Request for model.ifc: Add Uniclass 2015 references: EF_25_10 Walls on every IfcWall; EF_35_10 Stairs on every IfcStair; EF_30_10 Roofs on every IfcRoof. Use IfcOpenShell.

First a look at what the model holds.

```python
import ifcopenshell

model = ifcopenshell.open("model.ifc")
print(model.schema)
print("classifications:", [c.Name for c in model.by_type("IfcClassification")])
for ifc_class in ("IfcDoor", "IfcRoof", "IfcStair", "IfcWall", "IfcWindow"):
    print(ifc_class, len(model.by_type(ifc_class)))
```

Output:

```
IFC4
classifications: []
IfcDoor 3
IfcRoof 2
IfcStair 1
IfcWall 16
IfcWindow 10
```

```python
import ifcopenshell
import ifcopenshell.api.classification

model = ifcopenshell.open("model.ifc")

system = ifcopenshell.api.classification.add_classification(model, classification="Uniclass 2015")

codes = {
    "IfcWall": ("EF_25_10", "Walls"),
    "IfcStair": ("EF_35_10", "Stairs"),
    "IfcRoof": ("EF_30_10", "Roofs"),
}
for ifc_class, (code, name) in codes.items():
    products = model.by_type(ifc_class)
    ifcopenshell.api.classification.add_reference(
        model, products=products, classification=system, identification=code, name=name
    )
    print(code, len(products))

model.write("model-out.ifc")
```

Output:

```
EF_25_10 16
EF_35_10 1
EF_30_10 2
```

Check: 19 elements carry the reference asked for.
